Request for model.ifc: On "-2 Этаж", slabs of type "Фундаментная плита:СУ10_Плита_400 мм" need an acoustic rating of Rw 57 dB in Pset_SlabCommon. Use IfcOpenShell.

First a look at what the model holds.

```python
import ifcopenshell
import ifcopenshell.util.element

model = ifcopenshell.open("model.ifc")
print(model.schema)
storey = next(s for s in model.by_type("IfcBuildingStorey") if s.Name == "-2 Этаж")
slabs = [e for e in ifcopenshell.util.element.get_decomposition(storey) if e.is_a("IfcSlab")]
seen = {}
for e in slabs:
    element_type = ifcopenshell.util.element.get_type(e)
    key = (element_type.Name if element_type != e and element_type else None, ifcopenshell.util.element.get_pset(e, "Pset_SlabCommon", "AcousticRating"))
    seen[key] = seen.get(key, 0) + 1
for (name, value), count in sorted(seen.items(), key=str):
    print(count, "x", name, "|", value)
```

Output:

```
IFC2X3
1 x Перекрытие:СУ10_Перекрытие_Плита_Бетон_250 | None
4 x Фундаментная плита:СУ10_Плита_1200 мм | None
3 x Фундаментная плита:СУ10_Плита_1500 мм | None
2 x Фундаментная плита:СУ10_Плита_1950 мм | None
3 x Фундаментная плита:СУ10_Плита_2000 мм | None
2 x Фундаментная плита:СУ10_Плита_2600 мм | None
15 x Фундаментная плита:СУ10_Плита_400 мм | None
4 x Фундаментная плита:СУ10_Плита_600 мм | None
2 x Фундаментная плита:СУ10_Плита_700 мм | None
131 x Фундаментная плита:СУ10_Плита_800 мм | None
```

```python
import ifcopenshell
import ifcopenshell.api.pset
import ifcopenshell.util.element

model = ifcopenshell.open("model.ifc")

storey = next(s for s in model.by_type("IfcBuildingStorey") if s.Name == "-2 Этаж")
slabs = [e for e in ifcopenshell.util.element.get_decomposition(storey) if e.is_a("IfcSlab")]

count = 0
for e in slabs:
    element_type = ifcopenshell.util.element.get_type(e)
    if element_type in (None, e) or element_type.Name != "Фундаментная плита:СУ10_Плита_400 мм":
        continue
    # add_pset returns the element's existing set when there is one.
    pset = ifcopenshell.api.pset.add_pset(model, product=e, name="Pset_SlabCommon")
    ifcopenshell.api.pset.edit_pset(model, pset=pset, properties={"AcousticRating": "Rw 57 dB"})
    count += 1

print(count, "slabs updated")

model.write("model_v2.ifc")
```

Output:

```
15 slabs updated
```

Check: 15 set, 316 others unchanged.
